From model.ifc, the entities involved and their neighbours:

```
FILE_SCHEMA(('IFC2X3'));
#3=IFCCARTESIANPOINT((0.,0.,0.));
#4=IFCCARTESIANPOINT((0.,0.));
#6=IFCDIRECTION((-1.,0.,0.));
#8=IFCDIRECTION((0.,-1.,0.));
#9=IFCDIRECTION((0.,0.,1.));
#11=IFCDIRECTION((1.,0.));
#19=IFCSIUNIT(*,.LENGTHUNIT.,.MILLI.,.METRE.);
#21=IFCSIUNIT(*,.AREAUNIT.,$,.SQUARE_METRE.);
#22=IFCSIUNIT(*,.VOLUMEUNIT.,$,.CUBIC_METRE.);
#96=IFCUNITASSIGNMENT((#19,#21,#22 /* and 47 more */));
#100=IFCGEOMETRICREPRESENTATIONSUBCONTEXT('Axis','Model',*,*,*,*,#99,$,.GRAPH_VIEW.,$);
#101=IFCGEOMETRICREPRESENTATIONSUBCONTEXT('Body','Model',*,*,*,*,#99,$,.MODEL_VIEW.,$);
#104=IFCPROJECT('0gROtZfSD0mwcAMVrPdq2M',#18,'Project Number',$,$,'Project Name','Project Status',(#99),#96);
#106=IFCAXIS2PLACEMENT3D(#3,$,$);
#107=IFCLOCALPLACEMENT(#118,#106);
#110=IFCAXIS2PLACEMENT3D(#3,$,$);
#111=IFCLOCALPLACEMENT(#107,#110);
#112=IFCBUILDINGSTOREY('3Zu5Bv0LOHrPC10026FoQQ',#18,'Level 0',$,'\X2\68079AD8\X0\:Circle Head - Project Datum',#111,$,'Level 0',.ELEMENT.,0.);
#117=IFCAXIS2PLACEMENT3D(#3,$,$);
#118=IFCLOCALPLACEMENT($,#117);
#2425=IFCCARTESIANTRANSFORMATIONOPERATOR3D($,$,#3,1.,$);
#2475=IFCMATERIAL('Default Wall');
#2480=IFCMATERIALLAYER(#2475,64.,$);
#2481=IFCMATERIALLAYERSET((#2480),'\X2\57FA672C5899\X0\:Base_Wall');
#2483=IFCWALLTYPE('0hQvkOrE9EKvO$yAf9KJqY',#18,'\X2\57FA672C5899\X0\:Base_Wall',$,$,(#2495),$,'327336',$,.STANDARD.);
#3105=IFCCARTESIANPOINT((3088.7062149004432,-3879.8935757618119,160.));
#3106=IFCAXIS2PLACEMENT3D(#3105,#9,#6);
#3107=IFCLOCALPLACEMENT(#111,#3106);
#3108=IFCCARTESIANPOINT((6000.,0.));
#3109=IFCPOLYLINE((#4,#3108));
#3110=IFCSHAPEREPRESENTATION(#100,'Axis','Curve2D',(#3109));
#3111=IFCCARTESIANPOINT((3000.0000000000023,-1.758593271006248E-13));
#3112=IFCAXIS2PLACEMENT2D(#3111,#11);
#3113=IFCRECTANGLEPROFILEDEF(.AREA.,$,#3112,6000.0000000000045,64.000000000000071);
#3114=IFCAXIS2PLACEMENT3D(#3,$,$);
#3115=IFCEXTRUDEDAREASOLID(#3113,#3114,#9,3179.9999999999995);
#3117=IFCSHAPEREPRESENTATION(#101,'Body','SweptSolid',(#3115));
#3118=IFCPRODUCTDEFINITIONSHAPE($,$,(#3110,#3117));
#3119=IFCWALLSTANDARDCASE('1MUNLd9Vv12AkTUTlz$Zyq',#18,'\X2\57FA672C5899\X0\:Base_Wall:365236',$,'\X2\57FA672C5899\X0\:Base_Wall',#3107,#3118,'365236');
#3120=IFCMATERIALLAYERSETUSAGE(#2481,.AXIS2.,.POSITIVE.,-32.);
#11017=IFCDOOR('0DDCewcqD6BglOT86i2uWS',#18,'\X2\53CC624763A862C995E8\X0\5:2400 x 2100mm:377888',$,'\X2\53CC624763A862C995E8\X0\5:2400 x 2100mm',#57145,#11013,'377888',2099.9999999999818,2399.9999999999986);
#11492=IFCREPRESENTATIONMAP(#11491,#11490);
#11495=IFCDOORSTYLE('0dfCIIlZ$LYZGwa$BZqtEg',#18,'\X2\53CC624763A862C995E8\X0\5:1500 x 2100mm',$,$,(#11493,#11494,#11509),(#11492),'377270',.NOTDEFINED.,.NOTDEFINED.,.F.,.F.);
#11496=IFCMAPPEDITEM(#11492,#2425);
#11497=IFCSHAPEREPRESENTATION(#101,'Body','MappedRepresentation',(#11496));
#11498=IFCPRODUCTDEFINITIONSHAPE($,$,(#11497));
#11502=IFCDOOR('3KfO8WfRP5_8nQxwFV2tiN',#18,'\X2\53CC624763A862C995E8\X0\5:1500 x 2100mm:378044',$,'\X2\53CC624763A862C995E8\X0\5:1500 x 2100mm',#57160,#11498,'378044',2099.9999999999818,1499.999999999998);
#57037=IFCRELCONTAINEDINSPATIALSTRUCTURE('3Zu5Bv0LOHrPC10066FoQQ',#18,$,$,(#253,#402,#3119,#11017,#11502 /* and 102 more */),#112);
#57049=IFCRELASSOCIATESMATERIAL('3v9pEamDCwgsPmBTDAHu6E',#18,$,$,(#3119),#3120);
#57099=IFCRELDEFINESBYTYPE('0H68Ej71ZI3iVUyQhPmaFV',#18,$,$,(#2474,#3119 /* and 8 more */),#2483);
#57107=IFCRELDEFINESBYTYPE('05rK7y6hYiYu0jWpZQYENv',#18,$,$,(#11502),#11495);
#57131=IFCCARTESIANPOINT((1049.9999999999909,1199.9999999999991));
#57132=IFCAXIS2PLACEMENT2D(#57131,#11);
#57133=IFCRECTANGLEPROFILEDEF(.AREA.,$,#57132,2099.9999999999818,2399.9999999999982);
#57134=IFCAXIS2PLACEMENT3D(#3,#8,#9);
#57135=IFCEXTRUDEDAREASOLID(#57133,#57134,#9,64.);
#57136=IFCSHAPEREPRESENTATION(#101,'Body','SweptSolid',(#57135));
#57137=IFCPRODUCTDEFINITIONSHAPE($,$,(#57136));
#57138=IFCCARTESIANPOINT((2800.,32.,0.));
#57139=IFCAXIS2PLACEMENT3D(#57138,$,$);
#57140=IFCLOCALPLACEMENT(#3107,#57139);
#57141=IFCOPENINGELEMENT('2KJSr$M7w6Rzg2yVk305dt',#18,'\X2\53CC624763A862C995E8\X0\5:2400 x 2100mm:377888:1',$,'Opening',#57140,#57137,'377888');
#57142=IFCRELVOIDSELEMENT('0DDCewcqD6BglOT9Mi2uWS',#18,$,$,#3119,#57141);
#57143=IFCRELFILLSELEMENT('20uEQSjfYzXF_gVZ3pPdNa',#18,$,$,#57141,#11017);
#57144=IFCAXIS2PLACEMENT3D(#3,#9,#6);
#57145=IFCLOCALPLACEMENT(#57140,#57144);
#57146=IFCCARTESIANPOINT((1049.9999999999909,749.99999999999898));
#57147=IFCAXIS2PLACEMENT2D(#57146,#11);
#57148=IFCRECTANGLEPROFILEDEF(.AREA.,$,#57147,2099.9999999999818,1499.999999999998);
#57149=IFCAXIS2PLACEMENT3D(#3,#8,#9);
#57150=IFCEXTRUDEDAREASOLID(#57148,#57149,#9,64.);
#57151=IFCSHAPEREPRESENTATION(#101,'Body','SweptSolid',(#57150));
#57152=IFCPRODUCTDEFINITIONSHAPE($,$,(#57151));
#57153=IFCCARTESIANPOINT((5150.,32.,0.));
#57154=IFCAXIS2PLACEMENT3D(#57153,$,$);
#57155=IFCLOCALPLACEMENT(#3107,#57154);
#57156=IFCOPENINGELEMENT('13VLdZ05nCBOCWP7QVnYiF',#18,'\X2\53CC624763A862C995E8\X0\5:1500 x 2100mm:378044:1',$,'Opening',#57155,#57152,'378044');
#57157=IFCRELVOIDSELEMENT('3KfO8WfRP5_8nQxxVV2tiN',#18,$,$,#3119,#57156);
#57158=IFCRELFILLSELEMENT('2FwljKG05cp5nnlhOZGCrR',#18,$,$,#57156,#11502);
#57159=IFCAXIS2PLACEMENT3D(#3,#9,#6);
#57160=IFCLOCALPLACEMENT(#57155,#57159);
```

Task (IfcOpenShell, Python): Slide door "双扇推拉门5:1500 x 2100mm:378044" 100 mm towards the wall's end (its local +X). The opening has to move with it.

```python
import ifcopenshell
import ifcopenshell.api.geometry
import ifcopenshell.util.placement
import ifcopenshell.util.unit

model = ifcopenshell.open("model.ifc")
unit_scale = ifcopenshell.util.unit.calculate_unit_scale(model)

door = model.by_guid("3KfO8WfRP5_8nQxwFV2tiN")
opening = door.FillsVoids[0].RelatingOpeningElement
wall = opening.VoidsElements[0].RelatingBuildingElement

wall_matrix = ifcopenshell.util.placement.get_local_placement(wall.ObjectPlacement)
shift = wall_matrix[:3, 0] * 0.1 / unit_scale
before = ifcopenshell.util.placement.get_local_placement(door.ObjectPlacement)[:3, 3].copy()

# The door is placed relative to its opening, so it follows when the opening moves.
matrix = ifcopenshell.util.placement.get_local_placement(opening.ObjectPlacement)
matrix[:3, 3] += shift
ifcopenshell.api.geometry.edit_object_placement(
    model, product=opening, matrix=matrix, is_si=False, should_transform_children=True
)

after = ifcopenshell.util.placement.get_local_placement(door.ObjectPlacement)[:3, 3]
print("door moved by", (after - before).round(3) + 0.0)

model.write("model_v2.ifc")
```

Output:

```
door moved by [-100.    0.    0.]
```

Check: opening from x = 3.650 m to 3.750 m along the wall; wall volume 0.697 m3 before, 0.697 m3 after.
